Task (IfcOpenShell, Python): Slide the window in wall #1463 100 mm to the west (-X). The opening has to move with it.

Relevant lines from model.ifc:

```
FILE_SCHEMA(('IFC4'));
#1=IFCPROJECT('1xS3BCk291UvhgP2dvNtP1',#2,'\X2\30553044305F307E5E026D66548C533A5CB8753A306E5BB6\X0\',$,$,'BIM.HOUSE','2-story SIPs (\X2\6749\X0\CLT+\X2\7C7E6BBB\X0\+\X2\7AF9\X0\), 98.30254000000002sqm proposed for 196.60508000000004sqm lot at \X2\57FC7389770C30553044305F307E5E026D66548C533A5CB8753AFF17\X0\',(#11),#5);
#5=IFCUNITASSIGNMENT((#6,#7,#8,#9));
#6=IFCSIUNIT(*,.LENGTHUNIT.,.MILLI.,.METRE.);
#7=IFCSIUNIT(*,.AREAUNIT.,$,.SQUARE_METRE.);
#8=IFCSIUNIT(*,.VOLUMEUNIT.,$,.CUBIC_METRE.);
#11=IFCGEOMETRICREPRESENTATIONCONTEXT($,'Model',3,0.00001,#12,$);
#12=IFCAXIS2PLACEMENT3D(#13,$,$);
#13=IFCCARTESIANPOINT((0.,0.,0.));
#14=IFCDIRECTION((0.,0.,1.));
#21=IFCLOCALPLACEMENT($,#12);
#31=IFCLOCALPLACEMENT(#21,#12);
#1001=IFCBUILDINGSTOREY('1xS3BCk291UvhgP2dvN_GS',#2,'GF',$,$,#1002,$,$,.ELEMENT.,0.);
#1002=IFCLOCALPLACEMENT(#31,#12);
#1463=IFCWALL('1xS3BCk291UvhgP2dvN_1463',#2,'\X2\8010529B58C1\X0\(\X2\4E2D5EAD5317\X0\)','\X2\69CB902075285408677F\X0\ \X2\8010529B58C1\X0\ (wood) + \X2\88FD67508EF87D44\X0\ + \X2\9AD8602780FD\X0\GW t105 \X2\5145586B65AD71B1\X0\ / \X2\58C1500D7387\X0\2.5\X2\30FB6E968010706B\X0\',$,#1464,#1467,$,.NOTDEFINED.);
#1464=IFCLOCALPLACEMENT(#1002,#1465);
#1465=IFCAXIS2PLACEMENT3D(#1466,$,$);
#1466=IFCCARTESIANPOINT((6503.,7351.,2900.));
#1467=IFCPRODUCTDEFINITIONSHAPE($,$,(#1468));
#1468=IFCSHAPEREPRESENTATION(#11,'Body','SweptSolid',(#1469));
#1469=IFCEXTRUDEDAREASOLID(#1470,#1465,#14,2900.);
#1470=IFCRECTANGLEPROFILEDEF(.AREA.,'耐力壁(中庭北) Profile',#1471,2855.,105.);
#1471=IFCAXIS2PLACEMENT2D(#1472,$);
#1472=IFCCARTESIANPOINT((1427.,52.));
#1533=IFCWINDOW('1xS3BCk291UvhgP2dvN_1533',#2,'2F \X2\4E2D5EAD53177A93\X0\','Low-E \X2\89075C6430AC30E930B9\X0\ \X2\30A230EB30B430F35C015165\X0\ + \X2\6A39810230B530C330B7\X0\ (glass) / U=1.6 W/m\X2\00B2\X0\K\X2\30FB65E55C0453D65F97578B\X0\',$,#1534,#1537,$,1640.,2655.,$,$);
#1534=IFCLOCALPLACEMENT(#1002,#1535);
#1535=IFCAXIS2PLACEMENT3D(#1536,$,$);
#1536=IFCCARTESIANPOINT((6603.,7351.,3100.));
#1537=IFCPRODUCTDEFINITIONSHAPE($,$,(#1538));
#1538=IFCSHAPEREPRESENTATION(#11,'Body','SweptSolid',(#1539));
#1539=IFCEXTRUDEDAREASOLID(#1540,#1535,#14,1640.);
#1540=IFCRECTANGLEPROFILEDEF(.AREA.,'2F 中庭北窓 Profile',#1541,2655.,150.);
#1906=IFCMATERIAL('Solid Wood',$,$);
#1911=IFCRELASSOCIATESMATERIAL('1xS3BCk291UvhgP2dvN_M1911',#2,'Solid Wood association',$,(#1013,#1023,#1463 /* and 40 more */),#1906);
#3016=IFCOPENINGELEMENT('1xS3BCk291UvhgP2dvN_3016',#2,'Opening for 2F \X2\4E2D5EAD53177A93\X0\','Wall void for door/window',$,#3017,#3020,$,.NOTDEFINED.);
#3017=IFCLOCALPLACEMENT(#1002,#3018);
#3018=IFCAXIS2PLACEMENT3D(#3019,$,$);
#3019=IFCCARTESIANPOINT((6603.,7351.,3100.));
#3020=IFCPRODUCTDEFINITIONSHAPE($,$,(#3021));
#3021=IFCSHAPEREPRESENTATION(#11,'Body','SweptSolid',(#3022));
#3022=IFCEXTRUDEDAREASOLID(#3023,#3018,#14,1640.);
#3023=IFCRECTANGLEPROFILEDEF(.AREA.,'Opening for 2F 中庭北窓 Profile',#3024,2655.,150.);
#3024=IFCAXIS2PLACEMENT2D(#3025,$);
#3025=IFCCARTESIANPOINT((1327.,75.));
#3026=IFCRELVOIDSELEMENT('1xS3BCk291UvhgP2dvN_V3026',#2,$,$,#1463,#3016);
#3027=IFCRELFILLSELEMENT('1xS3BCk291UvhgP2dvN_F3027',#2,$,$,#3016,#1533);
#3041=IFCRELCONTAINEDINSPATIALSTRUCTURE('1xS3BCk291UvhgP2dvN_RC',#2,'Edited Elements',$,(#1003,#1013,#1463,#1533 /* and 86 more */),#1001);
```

```python
import ifcopenshell
import ifcopenshell.api.geometry
import ifcopenshell.util.placement
import ifcopenshell.util.unit

model = ifcopenshell.open("model.ifc")
unit_scale = ifcopenshell.util.unit.calculate_unit_scale(model)

window = model.by_guid("1xS3BCk291UvhgP2dvN_1533")
opening = window.FillsVoids[0].RelatingOpeningElement
wall = opening.VoidsElements[0].RelatingBuildingElement

wall_matrix = ifcopenshell.util.placement.get_local_placement(wall.ObjectPlacement)
shift = wall_matrix[:3, 0] * -0.1 / unit_scale
before = ifcopenshell.util.placement.get_local_placement(window.ObjectPlacement)[:3, 3].copy()

# The window is not placed relative to its opening, so move both.
for product in (opening, window):
    matrix = ifcopenshell.util.placement.get_local_placement(product.ObjectPlacement)
    matrix[:3, 3] += shift
    ifcopenshell.api.geometry.edit_object_placement(model, product=product, matrix=matrix, is_si=False)

after = ifcopenshell.util.placement.get_local_placement(window.ObjectPlacement)[:3, 3]
print("window moved by", (after - before).round(3) + 0.0)

model.write("model_rev.ifc")
```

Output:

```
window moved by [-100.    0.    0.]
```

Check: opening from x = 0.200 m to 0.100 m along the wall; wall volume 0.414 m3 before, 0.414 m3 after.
